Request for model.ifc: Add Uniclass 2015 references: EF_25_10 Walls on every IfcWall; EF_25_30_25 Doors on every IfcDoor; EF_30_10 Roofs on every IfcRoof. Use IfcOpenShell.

First a look at what the model holds.

```python
import ifcopenshell

model = ifcopenshell.open("model.ifc")
print(model.schema)
print("classifications:", [c.Name for c in model.by_type("IfcClassification")])
for ifc_class in ("IfcDoor", "IfcRoof", "IfcStair", "IfcWall", "IfcWindow"):
    print(ifc_class, len(model.by_type(ifc_class)))
```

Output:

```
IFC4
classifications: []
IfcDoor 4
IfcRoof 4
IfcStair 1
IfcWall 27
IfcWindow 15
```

```python
import ifcopenshell
import ifcopenshell.api.classification

model = ifcopenshell.open("model.ifc")

system = ifcopenshell.api.classification.add_classification(model, classification="Uniclass 2015")

codes = {
    "IfcWall": ("EF_25_10", "Walls"),
    "IfcDoor": ("EF_25_30_25", "Doors"),
    "IfcRoof": ("EF_30_10", "Roofs"),
}
for ifc_class, (code, name) in codes.items():
    products = model.by_type(ifc_class)
    ifcopenshell.api.classification.add_reference(
        model, products=products, classification=system, identification=code, name=name
    )
    print(code, len(products))

model.write("model-out.ifc")
```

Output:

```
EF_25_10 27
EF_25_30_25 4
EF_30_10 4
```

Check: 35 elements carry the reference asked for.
